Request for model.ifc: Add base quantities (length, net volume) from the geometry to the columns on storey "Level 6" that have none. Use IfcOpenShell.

First a look at what the model holds.

```python
import ifcopenshell
import ifcopenshell.util.element
import ifcopenshell.util.unit

model = ifcopenshell.open("model.ifc")
print(model.schema)
for unit_type in ("LENGTHUNIT", "AREAUNIT", "VOLUMEUNIT"):
    print(unit_type, ifcopenshell.util.unit.calculate_unit_scale(model, unit_type))
storey = next(s for s in model.by_type("IfcBuildingStorey") if s.Name == "Level 6")
columns = [e for e in ifcopenshell.util.element.get_decomposition(storey) if e.is_a("IfcColumn")]
for e in sorted(columns, key=lambda e: e.id()):
    print(e.id(), e.is_a(), e.Name, list(ifcopenshell.util.element.get_psets(e, qtos_only=True)), sep=" | ")
```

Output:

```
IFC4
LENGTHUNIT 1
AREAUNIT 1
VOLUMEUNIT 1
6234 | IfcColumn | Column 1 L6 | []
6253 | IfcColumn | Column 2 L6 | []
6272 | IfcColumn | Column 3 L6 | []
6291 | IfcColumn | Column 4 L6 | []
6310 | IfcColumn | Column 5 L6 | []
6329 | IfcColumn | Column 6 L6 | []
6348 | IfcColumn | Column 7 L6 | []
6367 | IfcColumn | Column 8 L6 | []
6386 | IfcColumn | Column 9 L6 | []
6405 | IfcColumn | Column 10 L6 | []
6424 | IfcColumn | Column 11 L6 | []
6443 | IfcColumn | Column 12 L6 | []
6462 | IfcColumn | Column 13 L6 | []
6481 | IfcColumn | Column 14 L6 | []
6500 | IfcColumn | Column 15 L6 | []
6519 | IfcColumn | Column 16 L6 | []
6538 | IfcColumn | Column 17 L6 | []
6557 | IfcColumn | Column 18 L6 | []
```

```python
import ifcopenshell
import ifcopenshell.api.pset
import ifcopenshell.geom
import ifcopenshell.util.element
import ifcopenshell.util.shape
import ifcopenshell.util.unit

model = ifcopenshell.open("model.ifc")
unit_scale = ifcopenshell.util.unit.calculate_unit_scale(model)
volume_scale = ifcopenshell.util.unit.calculate_unit_scale(model, "VOLUMEUNIT")
settings = ifcopenshell.geom.settings()

storey = next(s for s in model.by_type("IfcBuildingStorey") if s.Name == "Level 6")
columns = [e for e in ifcopenshell.util.element.get_decomposition(storey) if e.is_a("IfcColumn")]

for e in sorted(columns, key=lambda e: e.id()):
    if ifcopenshell.util.element.get_psets(e, qtos_only=True, should_inherit=False):
        continue
    # Geometry comes back in metres, in the element's own axes.
    shape = ifcopenshell.geom.create_shape(settings, e)
    values = {
        "Length": ifcopenshell.util.shape.get_z(shape.geometry) / unit_scale,
        "NetVolume": ifcopenshell.util.shape.get_volume(shape.geometry) / volume_scale,
    }
    qto = ifcopenshell.api.pset.add_qto(model, product=e, name="Qto_ColumnBaseQuantities")
    ifcopenshell.api.pset.edit_qto(model, qto=qto, properties=values)
    print(e.id(), {k: round(v, 3) for k, v in values.items()})

model.write("model_updated.ifc")
```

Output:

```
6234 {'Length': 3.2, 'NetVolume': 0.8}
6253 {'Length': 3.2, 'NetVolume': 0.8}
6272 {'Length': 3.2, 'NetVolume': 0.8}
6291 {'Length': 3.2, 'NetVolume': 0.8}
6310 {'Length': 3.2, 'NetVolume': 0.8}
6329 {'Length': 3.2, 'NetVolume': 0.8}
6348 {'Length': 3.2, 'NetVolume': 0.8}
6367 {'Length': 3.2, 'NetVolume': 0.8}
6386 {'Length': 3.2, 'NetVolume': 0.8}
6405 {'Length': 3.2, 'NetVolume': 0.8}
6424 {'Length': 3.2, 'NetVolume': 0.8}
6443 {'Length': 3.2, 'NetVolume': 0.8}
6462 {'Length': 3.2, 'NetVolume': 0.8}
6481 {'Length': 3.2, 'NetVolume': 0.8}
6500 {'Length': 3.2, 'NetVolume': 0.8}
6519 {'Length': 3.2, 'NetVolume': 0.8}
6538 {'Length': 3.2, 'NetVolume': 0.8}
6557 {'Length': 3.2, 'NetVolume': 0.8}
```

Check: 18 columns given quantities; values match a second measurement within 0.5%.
